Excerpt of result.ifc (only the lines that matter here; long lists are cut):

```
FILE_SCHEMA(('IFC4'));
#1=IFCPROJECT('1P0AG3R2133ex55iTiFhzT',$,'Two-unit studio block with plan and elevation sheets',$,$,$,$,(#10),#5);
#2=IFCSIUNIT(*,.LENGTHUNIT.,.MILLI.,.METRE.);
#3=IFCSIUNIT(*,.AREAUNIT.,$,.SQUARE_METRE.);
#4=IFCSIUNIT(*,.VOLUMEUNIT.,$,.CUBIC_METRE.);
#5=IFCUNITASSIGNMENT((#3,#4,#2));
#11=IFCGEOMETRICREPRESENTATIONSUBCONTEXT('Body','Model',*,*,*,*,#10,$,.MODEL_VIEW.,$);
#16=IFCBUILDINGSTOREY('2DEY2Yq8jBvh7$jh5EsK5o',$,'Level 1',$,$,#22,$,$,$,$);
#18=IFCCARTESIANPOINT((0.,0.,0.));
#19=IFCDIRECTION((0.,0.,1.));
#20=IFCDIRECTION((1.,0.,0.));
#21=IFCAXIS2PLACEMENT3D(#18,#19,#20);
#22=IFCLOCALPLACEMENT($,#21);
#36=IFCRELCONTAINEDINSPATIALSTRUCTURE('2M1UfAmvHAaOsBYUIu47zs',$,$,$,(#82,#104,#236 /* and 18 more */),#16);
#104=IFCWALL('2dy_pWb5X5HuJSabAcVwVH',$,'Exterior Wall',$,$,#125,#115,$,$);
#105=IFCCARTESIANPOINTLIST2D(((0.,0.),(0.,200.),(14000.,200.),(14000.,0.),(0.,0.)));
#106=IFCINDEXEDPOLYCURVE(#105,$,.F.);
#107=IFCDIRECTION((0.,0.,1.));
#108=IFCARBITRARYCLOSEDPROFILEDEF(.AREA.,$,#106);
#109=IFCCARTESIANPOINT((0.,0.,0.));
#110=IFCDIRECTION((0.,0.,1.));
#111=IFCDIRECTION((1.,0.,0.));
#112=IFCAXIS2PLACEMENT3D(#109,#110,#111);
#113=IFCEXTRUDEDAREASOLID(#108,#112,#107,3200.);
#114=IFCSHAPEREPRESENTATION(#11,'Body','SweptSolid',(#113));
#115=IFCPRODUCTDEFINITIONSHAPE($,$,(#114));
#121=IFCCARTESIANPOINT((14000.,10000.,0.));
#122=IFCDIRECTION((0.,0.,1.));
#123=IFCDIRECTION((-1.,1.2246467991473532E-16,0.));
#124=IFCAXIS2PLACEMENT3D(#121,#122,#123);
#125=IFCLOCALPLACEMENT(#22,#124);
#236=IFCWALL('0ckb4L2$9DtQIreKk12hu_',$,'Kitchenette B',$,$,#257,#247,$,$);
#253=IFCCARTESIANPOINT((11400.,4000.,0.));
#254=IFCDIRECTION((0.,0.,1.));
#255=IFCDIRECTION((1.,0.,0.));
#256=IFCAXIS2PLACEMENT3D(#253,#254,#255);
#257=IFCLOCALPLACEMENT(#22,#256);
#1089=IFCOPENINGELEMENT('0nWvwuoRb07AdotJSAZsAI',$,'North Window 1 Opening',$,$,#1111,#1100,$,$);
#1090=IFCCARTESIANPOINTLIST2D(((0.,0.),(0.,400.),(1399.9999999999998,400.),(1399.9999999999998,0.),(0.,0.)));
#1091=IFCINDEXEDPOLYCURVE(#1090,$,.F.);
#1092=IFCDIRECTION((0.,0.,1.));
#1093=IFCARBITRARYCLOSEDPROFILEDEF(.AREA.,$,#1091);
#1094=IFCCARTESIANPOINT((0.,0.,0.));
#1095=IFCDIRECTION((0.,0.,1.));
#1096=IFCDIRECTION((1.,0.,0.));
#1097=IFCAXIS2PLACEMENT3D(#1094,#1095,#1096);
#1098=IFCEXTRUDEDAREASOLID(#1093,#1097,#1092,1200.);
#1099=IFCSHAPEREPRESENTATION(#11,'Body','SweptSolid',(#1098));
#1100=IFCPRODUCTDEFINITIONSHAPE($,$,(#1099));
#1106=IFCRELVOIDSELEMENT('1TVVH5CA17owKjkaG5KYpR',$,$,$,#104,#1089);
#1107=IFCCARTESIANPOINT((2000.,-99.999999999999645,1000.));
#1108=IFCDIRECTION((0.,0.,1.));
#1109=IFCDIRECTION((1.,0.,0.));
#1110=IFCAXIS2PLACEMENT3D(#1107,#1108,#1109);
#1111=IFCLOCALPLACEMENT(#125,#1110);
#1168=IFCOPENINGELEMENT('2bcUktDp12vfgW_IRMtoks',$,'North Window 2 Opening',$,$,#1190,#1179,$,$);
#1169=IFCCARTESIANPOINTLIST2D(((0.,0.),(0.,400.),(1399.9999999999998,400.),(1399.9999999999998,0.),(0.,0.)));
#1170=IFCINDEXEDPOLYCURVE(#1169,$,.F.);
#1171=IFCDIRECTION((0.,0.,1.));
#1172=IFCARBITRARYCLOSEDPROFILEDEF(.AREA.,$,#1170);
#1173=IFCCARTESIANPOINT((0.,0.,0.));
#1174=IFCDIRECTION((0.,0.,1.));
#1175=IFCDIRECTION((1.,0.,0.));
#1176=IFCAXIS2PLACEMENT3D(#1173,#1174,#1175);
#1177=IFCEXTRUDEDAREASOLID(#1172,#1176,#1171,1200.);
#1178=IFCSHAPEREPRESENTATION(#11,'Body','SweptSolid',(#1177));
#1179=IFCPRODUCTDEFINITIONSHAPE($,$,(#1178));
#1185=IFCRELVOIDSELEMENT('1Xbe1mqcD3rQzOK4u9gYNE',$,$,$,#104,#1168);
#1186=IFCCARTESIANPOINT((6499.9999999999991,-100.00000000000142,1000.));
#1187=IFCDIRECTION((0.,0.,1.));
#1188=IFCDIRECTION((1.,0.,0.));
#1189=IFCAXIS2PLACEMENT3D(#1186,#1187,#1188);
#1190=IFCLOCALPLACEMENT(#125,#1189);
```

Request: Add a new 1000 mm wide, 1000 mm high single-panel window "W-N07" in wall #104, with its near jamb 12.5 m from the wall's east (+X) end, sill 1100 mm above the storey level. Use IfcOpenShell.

```python
import numpy as np
import ifcopenshell
import ifcopenshell.api.feature
import ifcopenshell.api.geometry
import ifcopenshell.api.root
import ifcopenshell.api.spatial
import ifcopenshell.geom
import ifcopenshell.util.element
import ifcopenshell.util.placement
import ifcopenshell.util.representation
import ifcopenshell.util.shape
import ifcopenshell.util.unit

model = ifcopenshell.open("result.ifc")
unit_scale = ifcopenshell.util.unit.calculate_unit_scale(model)
settings = ifcopenshell.geom.settings()


def volume(element):
    """Net volume in cubic metres, openings subtracted."""
    shape = ifcopenshell.geom.create_shape(settings, element)
    return ifcopenshell.util.shape.get_volume(shape.geometry)


wall = model.by_guid("2dy_pWb5X5HuJSabAcVwVH")
storey = ifcopenshell.util.element.get_container(wall, ifc_class="IfcBuildingStorey")
context = ifcopenshell.util.representation.get_context(model, "Model", "Body", "MODEL_VIEW")
before = volume(wall)

width, height, from_end, sill = 1, 1, 12.5, 1.1  # metres

# The wall runs along its own X axis, and the end named is its -X end.
wall_shape = ifcopenshell.geom.create_shape(settings, wall)
x, y, z = ifcopenshell.util.shape.get_vertices(wall_shape.geometry).T
start = x.min() + from_end
face, thickness = float(y.min()), float(y.max() - y.min())
wall_matrix = ifcopenshell.util.placement.get_local_placement(wall.ObjectPlacement)
level = ifcopenshell.util.placement.get_local_placement(storey.ObjectPlacement)[2, 3]


def in_wall(x, y):
    """Placement at x, y metres in the wall's axes, at sill height."""
    matrix = wall_matrix.copy()
    matrix[:, 3] = wall_matrix @ np.array([x / unit_scale, y / unit_scale, 0.0, 1.0])
    matrix[2, 3] = level + sill / unit_scale
    return matrix


# Opening: a box that overshoots both wall faces by 50 mm.
opening = ifcopenshell.api.root.create_entity(model, ifc_class="IfcOpeningElement", predefined_type="OPENING")
box = ifcopenshell.api.geometry.add_wall_representation(
    model, context=context, length=width, height=height, thickness=thickness + 0.1
)
ifcopenshell.api.geometry.assign_representation(model, product=opening, representation=box)
ifcopenshell.api.geometry.edit_object_placement(model, product=opening, matrix=in_wall(start, face - 0.05), is_si=False)
ifcopenshell.api.feature.add_feature(model, feature=opening, element=wall)

window = ifcopenshell.api.root.create_entity(model, ifc_class="IfcWindow", name="W-N07", predefined_type="WINDOW")
window.OverallWidth, window.OverallHeight = width / unit_scale, height / unit_scale
window.PartitioningType = "SINGLE_PANEL"
body = ifcopenshell.api.geometry.add_window_representation(
    model,
    context=context,
    overall_width=window.OverallWidth,
    overall_height=window.OverallHeight,
    partition_type="SINGLE_PANEL",
)
ifcopenshell.api.geometry.assign_representation(model, product=window, representation=body)
ifcopenshell.api.spatial.assign_container(model, products=[window], relating_structure=storey)
ifcopenshell.api.feature.add_filling(model, opening=opening, element=window)

# Centre the window in the wall's thickness.
ifcopenshell.api.geometry.edit_object_placement(model, product=window, matrix=in_wall(start, face), is_si=False)
window_shape = ifcopenshell.geom.create_shape(settings, window)
depth = ifcopenshell.util.shape.get_vertices(window_shape.geometry)[:, 1]
offset = face + thickness / 2 - (depth.min() + depth.max()) / 2
ifcopenshell.api.geometry.edit_object_placement(model, product=window, matrix=in_wall(start, offset), is_si=False)

after = volume(wall)

print(f"wall volume {before:.3f} -> {after:.3f} m3")

model.write("result_v2.ifc")
```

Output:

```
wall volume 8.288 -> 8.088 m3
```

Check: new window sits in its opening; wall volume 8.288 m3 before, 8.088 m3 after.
